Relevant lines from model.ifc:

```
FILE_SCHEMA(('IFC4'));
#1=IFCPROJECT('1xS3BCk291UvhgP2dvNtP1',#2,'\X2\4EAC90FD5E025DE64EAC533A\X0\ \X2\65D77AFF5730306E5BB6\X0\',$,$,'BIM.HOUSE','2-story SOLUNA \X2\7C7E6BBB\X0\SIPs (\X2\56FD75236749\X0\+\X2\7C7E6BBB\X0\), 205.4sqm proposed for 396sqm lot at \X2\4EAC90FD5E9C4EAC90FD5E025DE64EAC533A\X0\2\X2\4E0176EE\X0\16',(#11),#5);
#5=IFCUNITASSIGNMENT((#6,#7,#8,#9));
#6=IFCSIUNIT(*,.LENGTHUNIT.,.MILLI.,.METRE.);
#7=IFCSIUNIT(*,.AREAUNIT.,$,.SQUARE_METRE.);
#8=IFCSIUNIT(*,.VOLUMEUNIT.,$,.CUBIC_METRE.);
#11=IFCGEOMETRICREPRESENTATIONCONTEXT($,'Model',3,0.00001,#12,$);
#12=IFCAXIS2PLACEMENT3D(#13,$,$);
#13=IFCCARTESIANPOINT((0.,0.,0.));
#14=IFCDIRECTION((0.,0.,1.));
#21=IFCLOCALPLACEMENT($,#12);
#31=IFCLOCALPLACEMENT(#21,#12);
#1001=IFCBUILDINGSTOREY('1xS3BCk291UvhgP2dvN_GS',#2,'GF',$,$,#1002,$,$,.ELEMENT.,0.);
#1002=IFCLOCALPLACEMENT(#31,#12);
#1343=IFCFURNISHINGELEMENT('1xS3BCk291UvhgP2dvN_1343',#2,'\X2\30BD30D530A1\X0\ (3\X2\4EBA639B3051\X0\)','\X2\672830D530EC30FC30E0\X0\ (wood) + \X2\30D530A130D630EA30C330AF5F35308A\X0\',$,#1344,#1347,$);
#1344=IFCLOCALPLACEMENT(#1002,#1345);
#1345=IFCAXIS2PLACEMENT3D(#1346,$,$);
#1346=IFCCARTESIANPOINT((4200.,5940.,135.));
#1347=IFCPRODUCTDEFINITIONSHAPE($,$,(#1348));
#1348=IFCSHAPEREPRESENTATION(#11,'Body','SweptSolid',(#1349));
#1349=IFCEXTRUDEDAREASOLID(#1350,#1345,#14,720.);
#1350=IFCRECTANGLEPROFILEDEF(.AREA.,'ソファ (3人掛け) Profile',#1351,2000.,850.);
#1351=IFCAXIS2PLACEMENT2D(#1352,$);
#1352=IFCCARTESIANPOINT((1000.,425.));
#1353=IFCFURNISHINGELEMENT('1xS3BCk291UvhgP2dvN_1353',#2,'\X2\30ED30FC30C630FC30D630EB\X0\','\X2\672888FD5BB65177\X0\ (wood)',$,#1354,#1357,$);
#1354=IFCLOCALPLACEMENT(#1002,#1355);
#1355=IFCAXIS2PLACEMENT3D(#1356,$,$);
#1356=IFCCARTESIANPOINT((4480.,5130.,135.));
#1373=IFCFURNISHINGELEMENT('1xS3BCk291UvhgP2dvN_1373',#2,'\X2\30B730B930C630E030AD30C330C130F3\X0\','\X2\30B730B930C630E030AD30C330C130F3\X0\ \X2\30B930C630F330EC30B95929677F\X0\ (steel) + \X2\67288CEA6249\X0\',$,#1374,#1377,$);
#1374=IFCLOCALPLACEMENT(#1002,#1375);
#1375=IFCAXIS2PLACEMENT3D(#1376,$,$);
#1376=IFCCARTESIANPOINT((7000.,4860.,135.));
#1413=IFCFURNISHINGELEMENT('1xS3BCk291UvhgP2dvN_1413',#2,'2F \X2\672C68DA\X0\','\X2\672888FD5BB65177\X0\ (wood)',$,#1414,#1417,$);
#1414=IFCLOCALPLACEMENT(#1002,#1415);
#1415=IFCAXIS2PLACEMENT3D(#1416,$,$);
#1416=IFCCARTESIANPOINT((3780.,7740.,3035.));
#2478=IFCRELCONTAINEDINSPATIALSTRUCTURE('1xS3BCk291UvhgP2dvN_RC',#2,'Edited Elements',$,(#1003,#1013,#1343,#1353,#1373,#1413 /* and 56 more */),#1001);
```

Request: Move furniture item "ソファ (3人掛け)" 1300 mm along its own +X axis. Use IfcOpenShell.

```python
import ifcopenshell
import ifcopenshell.api.geometry
import ifcopenshell.util.placement

model = ifcopenshell.open("model.ifc")

item = model.by_guid("1xS3BCk291UvhgP2dvN_1343")
matrix = ifcopenshell.util.placement.get_local_placement(item.ObjectPlacement)
matrix[:3, 3] += matrix[:3, 0] * 1300.0
ifcopenshell.api.geometry.edit_object_placement(model, product=item, matrix=matrix, is_si=False)

print(ifcopenshell.util.placement.get_local_placement(item.ObjectPlacement).round(3) + 0.0)

model.write("model_v2.ifc")
```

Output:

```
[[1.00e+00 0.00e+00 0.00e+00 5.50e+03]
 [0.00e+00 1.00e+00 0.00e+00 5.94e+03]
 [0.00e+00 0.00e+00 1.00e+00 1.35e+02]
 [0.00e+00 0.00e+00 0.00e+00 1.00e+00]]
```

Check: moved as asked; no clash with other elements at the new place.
